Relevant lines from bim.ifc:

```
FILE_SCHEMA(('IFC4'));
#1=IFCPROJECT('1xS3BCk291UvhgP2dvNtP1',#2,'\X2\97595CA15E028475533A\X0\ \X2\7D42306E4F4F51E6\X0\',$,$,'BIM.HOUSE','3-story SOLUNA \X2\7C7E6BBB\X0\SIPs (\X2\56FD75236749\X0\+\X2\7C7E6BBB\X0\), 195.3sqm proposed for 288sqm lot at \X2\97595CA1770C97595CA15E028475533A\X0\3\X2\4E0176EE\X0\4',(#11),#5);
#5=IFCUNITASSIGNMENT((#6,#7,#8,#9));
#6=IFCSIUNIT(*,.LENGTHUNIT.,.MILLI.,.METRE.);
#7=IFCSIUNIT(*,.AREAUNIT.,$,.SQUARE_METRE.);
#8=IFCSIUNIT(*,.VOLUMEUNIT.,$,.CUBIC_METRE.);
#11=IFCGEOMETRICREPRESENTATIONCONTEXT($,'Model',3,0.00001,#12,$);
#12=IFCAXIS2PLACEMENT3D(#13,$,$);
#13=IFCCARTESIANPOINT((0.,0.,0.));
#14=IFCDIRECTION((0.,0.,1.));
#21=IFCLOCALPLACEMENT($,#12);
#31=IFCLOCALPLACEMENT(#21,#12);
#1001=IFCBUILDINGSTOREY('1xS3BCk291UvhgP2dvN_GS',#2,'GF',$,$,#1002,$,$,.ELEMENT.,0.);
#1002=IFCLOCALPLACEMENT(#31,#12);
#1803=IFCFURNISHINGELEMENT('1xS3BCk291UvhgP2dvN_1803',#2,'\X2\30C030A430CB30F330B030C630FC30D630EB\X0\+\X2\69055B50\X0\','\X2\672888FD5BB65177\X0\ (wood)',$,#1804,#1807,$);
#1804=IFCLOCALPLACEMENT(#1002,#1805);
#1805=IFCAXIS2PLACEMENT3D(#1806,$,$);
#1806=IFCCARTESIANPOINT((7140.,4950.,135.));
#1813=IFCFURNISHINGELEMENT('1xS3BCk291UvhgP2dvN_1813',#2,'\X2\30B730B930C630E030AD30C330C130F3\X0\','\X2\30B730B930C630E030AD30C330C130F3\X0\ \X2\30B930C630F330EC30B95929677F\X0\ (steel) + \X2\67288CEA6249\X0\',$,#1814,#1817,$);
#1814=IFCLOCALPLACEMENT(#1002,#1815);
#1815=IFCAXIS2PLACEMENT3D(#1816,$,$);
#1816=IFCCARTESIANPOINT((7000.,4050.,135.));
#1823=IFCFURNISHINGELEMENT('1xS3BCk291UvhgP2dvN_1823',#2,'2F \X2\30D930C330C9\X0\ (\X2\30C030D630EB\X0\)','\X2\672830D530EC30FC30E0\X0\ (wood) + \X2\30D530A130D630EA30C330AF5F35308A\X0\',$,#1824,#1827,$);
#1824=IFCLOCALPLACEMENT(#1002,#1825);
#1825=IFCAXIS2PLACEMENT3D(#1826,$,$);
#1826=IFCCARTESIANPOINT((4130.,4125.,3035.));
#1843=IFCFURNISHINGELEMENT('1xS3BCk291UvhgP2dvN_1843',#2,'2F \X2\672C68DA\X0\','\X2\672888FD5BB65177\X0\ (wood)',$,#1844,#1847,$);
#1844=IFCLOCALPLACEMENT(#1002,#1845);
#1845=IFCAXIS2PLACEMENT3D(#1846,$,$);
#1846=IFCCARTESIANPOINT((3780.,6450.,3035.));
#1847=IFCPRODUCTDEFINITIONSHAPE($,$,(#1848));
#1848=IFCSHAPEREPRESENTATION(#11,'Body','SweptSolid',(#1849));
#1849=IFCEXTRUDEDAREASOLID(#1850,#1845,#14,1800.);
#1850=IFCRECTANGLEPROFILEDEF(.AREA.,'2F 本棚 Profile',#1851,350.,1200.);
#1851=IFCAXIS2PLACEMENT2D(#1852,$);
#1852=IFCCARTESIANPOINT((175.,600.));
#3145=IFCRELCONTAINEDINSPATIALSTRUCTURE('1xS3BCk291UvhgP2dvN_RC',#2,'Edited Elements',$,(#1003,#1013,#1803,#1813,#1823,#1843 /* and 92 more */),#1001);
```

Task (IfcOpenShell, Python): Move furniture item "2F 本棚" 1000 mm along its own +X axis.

```python
import ifcopenshell
import ifcopenshell.api.geometry
import ifcopenshell.util.placement
import ifcopenshell.util.unit

model = ifcopenshell.open("bim.ifc")
unit_scale = ifcopenshell.util.unit.calculate_unit_scale(model)

item = model.by_id(1843)
matrix = ifcopenshell.util.placement.get_local_placement(item.ObjectPlacement)
matrix[:3, 3] += matrix[:3, 0] * 1 / unit_scale
ifcopenshell.api.geometry.edit_object_placement(model, product=item, matrix=matrix, is_si=False)

print(ifcopenshell.util.placement.get_local_placement(item.ObjectPlacement).round(3) + 0.0)

model.write("bim_rev.ifc")
```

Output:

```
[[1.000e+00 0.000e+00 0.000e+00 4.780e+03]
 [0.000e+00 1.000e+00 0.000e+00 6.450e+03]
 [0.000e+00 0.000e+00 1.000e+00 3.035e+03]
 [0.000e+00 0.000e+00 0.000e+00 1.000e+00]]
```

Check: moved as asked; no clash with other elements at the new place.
